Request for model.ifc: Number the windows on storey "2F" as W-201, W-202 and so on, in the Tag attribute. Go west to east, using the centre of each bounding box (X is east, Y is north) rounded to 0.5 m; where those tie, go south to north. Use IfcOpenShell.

First a look at what the model holds.

```python
import ifcopenshell
import ifcopenshell.util.element
import ifcopenshell.util.placement

model = ifcopenshell.open("model.ifc")
print(model.schema)
storey = next(s for s in model.by_type("IfcBuildingStorey") if s.Name == "2F")
windows = [e for e in ifcopenshell.util.element.get_decomposition(storey) if e.is_a("IfcWindow")]
for e in sorted(windows, key=lambda e: e.id()):
    origin = ifcopenshell.util.placement.get_local_placement(e.ObjectPlacement)[:3, 3]
    print(e.id(), e.Tag, e.Name, origin.round(2) + 0.0, sep=" | ")
```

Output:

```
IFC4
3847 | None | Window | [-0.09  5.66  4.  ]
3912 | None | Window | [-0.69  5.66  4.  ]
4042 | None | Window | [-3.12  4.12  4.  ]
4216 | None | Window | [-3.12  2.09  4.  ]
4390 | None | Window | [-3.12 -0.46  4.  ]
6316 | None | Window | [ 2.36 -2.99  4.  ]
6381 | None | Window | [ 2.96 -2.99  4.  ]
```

```python
import ifcopenshell
import ifcopenshell.geom
import ifcopenshell.util.element
import ifcopenshell.util.shape

model = ifcopenshell.open("model.ifc")
settings = ifcopenshell.geom.settings()
settings.set("use-world-coords", True)


def centre(element):
    shape = ifcopenshell.geom.create_shape(settings, element)
    return ifcopenshell.util.shape.get_bbox_centroid(shape.geometry)


storey = next(s for s in model.by_type("IfcBuildingStorey") if s.Name == "2F")
windows = [e for e in ifcopenshell.util.element.get_decomposition(storey) if e.is_a("IfcWindow")]

# Insertion points can sit at a corner or the storey origin, so sort by the geometry (in metres).
centres = {e: centre(e) for e in windows}
windows.sort(key=lambda e: (round(centres[e][0] / 0.5), centres[e][1]))

for i, e in enumerate(windows, start=1):
    number = f"W-2{i:02d}"
    e.Tag = number
    print(e.id(), number)

model.write("model-out.ifc")
```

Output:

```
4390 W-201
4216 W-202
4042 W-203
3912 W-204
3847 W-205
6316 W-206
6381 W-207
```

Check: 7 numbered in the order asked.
